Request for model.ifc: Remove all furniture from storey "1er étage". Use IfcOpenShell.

First a look at what the model holds.

```python
import ifcopenshell
import ifcopenshell.util.element

model = ifcopenshell.open("model.ifc")
print(model.schema)
storey = next(s for s in model.by_type("IfcBuildingStorey") if s.Name == "1er étage")
furniture = [e for e in ifcopenshell.util.element.get_decomposition(storey) if e.is_a("IfcFurnishingElement")]
seen = {}
for e in furniture:
    element_type = ifcopenshell.util.element.get_type(e)
    name = element_type.Name if element_type not in (None, e) else None
    seen[name] = seen.get(name, 0) + 1
for name, count in sorted(seen.items(), key=str):
    print(count, "x", name)
```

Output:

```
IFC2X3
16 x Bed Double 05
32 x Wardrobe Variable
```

```python
import ifcopenshell
import ifcopenshell.api.root
import ifcopenshell.util.element

model = ifcopenshell.open("model.ifc")

storey = next(s for s in model.by_type("IfcBuildingStorey") if s.Name == "1er étage")
furniture = [e for e in ifcopenshell.util.element.get_decomposition(storey) if e.is_a("IfcFurnishingElement")]

for e in furniture:
    ifcopenshell.api.root.remove_product(model, product=e)
print(len(furniture), "removed")

model.write("model_v2.ifc")
```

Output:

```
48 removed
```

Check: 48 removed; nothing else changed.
